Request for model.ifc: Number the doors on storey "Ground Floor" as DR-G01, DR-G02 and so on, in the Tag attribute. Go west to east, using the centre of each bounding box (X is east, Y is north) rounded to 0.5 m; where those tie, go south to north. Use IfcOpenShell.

First a look at what the model holds.

```python
import ifcopenshell
import ifcopenshell.util.element
import ifcopenshell.util.placement

model = ifcopenshell.open("model.ifc")
print(model.schema)
storey = next(s for s in model.by_type("IfcBuildingStorey") if s.Name == "Ground Floor")
doors = [e for e in ifcopenshell.util.element.get_decomposition(storey) if e.is_a("IfcDoor")]
for e in sorted(doors, key=lambda e: e.id()):
    origin = ifcopenshell.util.placement.get_local_placement(e.ObjectPlacement)[:3, 3]
    print(e.id(), e.Tag, e.Name, origin.round(2) + 0.0, sep=" | ")
```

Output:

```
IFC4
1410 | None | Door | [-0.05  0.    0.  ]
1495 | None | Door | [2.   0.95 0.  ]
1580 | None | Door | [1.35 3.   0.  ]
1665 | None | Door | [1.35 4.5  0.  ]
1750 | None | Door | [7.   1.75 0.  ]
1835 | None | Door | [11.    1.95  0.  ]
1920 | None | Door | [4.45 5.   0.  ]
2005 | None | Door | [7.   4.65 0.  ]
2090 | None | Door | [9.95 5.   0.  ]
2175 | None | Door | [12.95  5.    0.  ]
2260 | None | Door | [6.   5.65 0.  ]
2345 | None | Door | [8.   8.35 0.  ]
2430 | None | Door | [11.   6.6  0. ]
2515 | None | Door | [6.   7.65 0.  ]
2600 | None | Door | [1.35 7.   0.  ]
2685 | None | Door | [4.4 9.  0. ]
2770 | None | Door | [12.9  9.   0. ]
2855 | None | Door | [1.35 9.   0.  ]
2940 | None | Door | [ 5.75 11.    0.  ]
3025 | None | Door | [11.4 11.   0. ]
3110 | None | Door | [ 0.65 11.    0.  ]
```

```python
import ifcopenshell
import ifcopenshell.geom
import ifcopenshell.util.element
import ifcopenshell.util.shape

model = ifcopenshell.open("model.ifc")
settings = ifcopenshell.geom.settings()
settings.set("use-world-coords", True)


def centre(element):
    shape = ifcopenshell.geom.create_shape(settings, element)
    return ifcopenshell.util.shape.get_bbox_centroid(shape.geometry)


storey = next(s for s in model.by_type("IfcBuildingStorey") if s.Name == "Ground Floor")
doors = [e for e in ifcopenshell.util.element.get_decomposition(storey) if e.is_a("IfcDoor")]

# Insertion points can sit at a corner or the storey origin, so sort by the geometry (in metres).
centres = {e: centre(e) for e in doors}
doors.sort(key=lambda e: (round(centres[e][0] / 0.5), centres[e][1]))

for i, e in enumerate(doors, start=1):
    number = f"DR-G{i:02d}"
    e.Tag = number
    print(e.id(), number)

model.write("model_v2.ifc")
```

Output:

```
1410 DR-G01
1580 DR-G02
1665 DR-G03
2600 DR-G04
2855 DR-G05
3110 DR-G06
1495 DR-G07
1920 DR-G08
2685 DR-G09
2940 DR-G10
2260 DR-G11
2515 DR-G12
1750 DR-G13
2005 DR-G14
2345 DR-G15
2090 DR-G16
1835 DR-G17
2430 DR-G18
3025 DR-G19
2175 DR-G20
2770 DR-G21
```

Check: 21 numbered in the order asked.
